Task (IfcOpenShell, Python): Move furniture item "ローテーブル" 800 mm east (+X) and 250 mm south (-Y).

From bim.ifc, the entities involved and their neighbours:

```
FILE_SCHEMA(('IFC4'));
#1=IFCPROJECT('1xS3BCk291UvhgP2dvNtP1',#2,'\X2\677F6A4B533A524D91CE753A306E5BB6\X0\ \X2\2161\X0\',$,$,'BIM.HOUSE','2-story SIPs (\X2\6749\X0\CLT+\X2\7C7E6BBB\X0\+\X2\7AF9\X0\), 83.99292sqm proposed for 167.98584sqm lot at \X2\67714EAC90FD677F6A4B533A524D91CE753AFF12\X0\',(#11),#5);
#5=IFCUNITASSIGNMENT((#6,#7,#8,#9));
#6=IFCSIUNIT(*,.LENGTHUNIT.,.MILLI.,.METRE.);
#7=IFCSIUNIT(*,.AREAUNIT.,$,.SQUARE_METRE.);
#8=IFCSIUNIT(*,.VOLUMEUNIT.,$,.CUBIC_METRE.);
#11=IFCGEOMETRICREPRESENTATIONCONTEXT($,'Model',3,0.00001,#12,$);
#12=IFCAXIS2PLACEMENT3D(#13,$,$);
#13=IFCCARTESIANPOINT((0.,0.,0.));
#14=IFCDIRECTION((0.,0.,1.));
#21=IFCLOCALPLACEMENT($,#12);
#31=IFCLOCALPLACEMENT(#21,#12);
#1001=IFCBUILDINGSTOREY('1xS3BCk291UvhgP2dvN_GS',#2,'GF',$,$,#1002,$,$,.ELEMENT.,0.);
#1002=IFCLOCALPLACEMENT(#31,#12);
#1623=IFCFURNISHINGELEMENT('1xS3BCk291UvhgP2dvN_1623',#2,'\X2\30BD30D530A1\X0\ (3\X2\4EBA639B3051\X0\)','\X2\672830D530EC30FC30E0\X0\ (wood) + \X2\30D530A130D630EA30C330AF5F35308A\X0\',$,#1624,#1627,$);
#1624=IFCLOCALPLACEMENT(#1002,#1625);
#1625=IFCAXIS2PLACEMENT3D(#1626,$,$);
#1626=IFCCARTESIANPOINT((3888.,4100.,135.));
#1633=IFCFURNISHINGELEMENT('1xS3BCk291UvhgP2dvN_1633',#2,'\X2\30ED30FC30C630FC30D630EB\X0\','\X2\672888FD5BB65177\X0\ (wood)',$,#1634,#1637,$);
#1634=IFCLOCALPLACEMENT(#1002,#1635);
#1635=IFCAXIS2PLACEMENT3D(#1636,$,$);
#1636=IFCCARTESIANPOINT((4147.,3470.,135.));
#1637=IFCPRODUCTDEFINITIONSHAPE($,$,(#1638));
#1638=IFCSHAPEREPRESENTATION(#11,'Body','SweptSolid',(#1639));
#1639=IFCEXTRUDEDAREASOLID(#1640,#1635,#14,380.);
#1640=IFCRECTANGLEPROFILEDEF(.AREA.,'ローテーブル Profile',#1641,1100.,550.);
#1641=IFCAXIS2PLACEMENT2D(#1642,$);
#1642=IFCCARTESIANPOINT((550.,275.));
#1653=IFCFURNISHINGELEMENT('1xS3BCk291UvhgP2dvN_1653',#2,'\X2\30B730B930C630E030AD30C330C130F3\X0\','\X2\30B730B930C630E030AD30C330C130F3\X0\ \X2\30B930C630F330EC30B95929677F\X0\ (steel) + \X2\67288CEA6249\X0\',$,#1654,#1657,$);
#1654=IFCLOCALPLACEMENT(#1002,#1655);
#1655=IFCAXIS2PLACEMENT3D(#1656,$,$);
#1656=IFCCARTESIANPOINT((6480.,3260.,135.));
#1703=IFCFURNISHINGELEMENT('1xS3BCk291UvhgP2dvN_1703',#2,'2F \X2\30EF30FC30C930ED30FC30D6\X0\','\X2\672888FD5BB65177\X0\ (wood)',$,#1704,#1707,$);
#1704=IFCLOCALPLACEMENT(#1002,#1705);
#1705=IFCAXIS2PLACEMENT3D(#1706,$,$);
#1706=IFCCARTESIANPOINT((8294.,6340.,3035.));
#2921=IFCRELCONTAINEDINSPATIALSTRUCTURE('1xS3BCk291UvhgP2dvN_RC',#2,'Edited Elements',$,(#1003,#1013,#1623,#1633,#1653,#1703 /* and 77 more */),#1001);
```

```python
import ifcopenshell
import ifcopenshell.api.geometry
import ifcopenshell.util.placement

model = ifcopenshell.open("bim.ifc")

item = model.by_guid("1xS3BCk291UvhgP2dvN_1633")
matrix = ifcopenshell.util.placement.get_local_placement(item.ObjectPlacement)
matrix[0, 3] += 800.0
matrix[1, 3] -= 250.0
ifcopenshell.api.geometry.edit_object_placement(model, product=item, matrix=matrix, is_si=False)

print(ifcopenshell.util.placement.get_local_placement(item.ObjectPlacement).round(3) + 0.0)

model.write("bim-out.ifc")
```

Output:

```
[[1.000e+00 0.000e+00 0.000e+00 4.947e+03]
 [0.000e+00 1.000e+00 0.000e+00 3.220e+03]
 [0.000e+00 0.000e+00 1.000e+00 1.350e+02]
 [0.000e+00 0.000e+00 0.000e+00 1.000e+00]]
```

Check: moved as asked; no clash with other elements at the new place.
